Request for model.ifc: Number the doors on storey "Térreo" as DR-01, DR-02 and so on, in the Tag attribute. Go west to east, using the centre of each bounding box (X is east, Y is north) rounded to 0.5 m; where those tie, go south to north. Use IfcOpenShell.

First a look at what the model holds.

```python
import ifcopenshell
import ifcopenshell.util.element
import ifcopenshell.util.placement

model = ifcopenshell.open("model.ifc")
print(model.schema)
storey = next(s for s in model.by_type("IfcBuildingStorey") if s.Name == "Térreo")
doors = [e for e in ifcopenshell.util.element.get_decomposition(storey) if e.is_a("IfcDoor")]
for e in sorted(doors, key=lambda e: e.id()):
    origin = ifcopenshell.util.placement.get_local_placement(e.ObjectPlacement)[:3, 3]
    print(e.id(), e.Tag, e.Name, origin.round(2) + 0.0, sep=" | ")
```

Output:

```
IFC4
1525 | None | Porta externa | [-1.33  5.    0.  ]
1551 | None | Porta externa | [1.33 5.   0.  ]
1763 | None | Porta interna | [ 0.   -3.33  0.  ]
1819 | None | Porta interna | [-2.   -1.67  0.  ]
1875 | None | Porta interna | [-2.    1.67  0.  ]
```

```python
import ifcopenshell
import ifcopenshell.geom
import ifcopenshell.util.element
import ifcopenshell.util.shape

model = ifcopenshell.open("model.ifc")
settings = ifcopenshell.geom.settings()
settings.set("use-world-coords", True)


def centre(element):
    shape = ifcopenshell.geom.create_shape(settings, element)
    return ifcopenshell.util.shape.get_bbox_centroid(shape.geometry)


storey = next(s for s in model.by_type("IfcBuildingStorey") if s.Name == "Térreo")
doors = [e for e in ifcopenshell.util.element.get_decomposition(storey) if e.is_a("IfcDoor")]

# Insertion points can sit at a corner or the storey origin, so sort by the geometry (in metres).
centres = {e: centre(e) for e in doors}
doors.sort(key=lambda e: (round(centres[e][0] / 0.5), centres[e][1]))

for i, e in enumerate(doors, start=1):
    number = f"DR-{i:02d}"
    e.Tag = number
    print(e.id(), number)

model.write("model_edited.ifc")
```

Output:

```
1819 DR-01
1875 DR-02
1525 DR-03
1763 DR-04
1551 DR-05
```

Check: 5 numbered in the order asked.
